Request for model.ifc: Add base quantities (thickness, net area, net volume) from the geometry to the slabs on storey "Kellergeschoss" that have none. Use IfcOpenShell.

First a look at what the model holds.

```python
import ifcopenshell
import ifcopenshell.util.element
import ifcopenshell.util.unit

model = ifcopenshell.open("model.ifc")
print(model.schema)
for unit_type in ("LENGTHUNIT", "AREAUNIT", "VOLUMEUNIT"):
    print(unit_type, ifcopenshell.util.unit.calculate_unit_scale(model, unit_type))
storey = next(s for s in model.by_type("IfcBuildingStorey") if s.Name == "Kellergeschoss")
slabs = [e for e in ifcopenshell.util.element.get_decomposition(storey) if e.is_a("IfcSlab")]
for e in sorted(slabs, key=lambda e: e.id()):
    print(e.id(), e.is_a(), e.Name, list(ifcopenshell.util.element.get_psets(e, qtos_only=True)), sep=" | ")
```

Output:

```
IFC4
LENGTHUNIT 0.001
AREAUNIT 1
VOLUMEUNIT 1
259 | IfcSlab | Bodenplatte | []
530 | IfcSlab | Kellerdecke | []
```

```python
import ifcopenshell
import ifcopenshell.api.pset
import ifcopenshell.geom
import ifcopenshell.util.element
import ifcopenshell.util.shape
import ifcopenshell.util.unit

model = ifcopenshell.open("model.ifc")
unit_scale = ifcopenshell.util.unit.calculate_unit_scale(model)
area_scale = ifcopenshell.util.unit.calculate_unit_scale(model, "AREAUNIT")
volume_scale = ifcopenshell.util.unit.calculate_unit_scale(model, "VOLUMEUNIT")
settings = ifcopenshell.geom.settings()

storey = next(s for s in model.by_type("IfcBuildingStorey") if s.Name == "Kellergeschoss")
slabs = [e for e in ifcopenshell.util.element.get_decomposition(storey) if e.is_a("IfcSlab")]

for e in sorted(slabs, key=lambda e: e.id()):
    if ifcopenshell.util.element.get_psets(e, qtos_only=True, should_inherit=False):
        continue
    # Geometry comes back in metres, in the element's own axes.
    shape = ifcopenshell.geom.create_shape(settings, e)
    values = {
        "Width": ifcopenshell.util.shape.get_z(shape.geometry) / unit_scale,
        "NetArea": ifcopenshell.util.shape.get_footprint_area(shape.geometry) / area_scale,
        "NetVolume": ifcopenshell.util.shape.get_volume(shape.geometry) / volume_scale,
    }
    qto = ifcopenshell.api.pset.add_qto(model, product=e, name="Qto_SlabBaseQuantities")
    ifcopenshell.api.pset.edit_qto(model, qto=qto, properties=values)
    print(e.id(), {k: round(v, 3) for k, v in values.items()})

model.write("model_edited.ifc")
```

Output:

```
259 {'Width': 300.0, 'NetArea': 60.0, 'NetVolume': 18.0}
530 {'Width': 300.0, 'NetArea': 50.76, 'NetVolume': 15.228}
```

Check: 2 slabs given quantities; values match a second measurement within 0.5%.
